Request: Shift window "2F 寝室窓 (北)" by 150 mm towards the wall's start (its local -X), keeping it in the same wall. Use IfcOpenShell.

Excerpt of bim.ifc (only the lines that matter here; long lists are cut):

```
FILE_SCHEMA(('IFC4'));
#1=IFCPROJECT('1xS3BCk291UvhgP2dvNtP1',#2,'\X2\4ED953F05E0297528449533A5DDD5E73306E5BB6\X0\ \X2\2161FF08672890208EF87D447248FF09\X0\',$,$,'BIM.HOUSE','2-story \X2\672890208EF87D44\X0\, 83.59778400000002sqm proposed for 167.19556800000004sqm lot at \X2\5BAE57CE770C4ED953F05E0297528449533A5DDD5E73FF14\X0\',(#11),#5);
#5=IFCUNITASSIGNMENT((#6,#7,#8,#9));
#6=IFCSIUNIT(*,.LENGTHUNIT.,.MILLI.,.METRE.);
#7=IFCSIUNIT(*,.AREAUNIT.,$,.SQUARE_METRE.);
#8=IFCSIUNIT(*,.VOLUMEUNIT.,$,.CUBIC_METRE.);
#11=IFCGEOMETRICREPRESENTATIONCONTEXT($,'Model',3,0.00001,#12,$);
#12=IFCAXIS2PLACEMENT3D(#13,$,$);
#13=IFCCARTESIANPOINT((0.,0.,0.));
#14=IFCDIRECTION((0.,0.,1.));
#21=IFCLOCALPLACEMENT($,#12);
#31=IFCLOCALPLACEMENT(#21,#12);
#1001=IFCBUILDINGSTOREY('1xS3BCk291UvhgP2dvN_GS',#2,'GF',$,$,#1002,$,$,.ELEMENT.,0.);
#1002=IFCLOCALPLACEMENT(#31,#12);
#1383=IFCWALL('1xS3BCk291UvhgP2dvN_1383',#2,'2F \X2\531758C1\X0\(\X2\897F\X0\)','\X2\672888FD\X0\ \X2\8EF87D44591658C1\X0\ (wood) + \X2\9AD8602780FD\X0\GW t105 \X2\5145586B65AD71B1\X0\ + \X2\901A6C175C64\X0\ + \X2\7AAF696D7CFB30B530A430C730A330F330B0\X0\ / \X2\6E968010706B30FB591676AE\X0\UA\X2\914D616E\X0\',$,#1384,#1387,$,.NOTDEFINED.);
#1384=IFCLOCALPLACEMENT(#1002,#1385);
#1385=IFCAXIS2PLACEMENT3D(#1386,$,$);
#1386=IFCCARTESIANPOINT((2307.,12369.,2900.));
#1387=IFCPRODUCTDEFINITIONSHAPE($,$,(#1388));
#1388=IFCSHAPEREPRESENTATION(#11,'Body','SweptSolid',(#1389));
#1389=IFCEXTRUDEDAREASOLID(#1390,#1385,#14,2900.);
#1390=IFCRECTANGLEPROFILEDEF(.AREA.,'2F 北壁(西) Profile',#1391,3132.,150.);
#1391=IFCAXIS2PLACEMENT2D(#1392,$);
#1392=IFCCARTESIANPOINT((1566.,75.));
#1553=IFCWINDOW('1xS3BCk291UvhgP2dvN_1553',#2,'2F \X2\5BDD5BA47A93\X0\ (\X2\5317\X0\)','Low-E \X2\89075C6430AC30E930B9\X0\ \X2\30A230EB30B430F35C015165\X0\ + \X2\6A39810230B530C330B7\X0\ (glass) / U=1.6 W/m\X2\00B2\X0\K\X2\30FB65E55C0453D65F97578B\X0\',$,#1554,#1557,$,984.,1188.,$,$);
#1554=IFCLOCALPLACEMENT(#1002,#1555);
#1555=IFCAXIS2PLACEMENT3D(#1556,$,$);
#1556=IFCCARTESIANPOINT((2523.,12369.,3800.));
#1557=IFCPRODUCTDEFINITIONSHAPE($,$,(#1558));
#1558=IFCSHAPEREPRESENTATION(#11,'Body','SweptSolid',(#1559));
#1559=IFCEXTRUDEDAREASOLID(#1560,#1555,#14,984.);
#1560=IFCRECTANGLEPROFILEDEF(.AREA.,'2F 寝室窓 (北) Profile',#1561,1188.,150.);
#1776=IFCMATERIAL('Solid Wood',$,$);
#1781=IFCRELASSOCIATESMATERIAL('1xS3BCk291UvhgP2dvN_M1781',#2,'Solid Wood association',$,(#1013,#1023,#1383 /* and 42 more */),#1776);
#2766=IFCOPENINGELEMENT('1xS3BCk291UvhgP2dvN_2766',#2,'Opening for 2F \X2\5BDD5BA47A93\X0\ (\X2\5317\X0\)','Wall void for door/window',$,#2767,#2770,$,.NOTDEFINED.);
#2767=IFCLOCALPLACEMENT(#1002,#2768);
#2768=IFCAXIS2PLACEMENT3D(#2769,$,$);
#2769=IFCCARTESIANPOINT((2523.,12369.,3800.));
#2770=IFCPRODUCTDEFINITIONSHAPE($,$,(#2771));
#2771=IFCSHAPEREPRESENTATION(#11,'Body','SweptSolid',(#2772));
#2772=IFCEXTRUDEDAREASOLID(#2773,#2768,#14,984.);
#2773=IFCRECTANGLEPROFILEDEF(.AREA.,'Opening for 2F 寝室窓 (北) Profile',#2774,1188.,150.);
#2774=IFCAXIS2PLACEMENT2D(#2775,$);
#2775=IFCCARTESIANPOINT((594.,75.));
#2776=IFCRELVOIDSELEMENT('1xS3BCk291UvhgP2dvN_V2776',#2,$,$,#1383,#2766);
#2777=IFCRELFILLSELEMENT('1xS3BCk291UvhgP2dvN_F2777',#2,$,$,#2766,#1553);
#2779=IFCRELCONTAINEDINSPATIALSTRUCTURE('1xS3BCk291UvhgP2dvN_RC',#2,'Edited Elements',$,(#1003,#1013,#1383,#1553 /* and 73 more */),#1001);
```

```python
import ifcopenshell
import ifcopenshell.api.geometry
import ifcopenshell.util.placement

model = ifcopenshell.open("bim.ifc")

window = model.by_id(1553)
opening = window.FillsVoids[0].RelatingOpeningElement
wall = opening.VoidsElements[0].RelatingBuildingElement

wall_matrix = ifcopenshell.util.placement.get_local_placement(wall.ObjectPlacement)
shift = wall_matrix[:3, 0] * -150.0
before = ifcopenshell.util.placement.get_local_placement(window.ObjectPlacement)[:3, 3].copy()

# The window is not placed relative to its opening, so move both.
for product in (opening, window):
    matrix = ifcopenshell.util.placement.get_local_placement(product.ObjectPlacement)
    matrix[:3, 3] += shift
    ifcopenshell.api.geometry.edit_object_placement(model, product=product, matrix=matrix, is_si=False)

after = ifcopenshell.util.placement.get_local_placement(window.ObjectPlacement)[:3, 3]
print("window moved by", (after - before).round(3) + 0.0)

model.write("bim_v2.ifc")
```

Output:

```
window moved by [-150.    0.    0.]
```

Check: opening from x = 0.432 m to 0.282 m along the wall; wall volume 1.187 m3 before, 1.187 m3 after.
